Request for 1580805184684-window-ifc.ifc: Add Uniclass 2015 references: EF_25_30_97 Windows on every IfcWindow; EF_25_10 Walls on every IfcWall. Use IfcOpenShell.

First a look at what the model holds.

```python
import ifcopenshell

model = ifcopenshell.open("1580805184684-window-ifc.ifc")
print(model.schema)
print("classifications:", [c.Name for c in model.by_type("IfcClassification")])
for ifc_class in ("IfcDoor", "IfcRoof", "IfcStair", "IfcWall", "IfcWindow"):
    print(ifc_class, len(model.by_type(ifc_class)))
```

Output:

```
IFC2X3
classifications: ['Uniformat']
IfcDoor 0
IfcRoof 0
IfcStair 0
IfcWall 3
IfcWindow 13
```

```python
import ifcopenshell
import ifcopenshell.api.classification

model = ifcopenshell.open("1580805184684-window-ifc.ifc")

# IFC2X3 requires Source and Edition and has no link from the project to the system.
system = model.create_entity("IfcClassification", Source="NBS", Edition="2015", Name="Uniclass 2015")

codes = {
    "IfcWindow": ("EF_25_30_97", "Windows"),
    "IfcWall": ("EF_25_10", "Walls"),
}
for ifc_class, (code, name) in codes.items():
    products = model.by_type(ifc_class)
    ifcopenshell.api.classification.add_reference(
        model, products=products, classification=system, identification=code, name=name
    )
    print(code, len(products))

model.write("1580805184684-window-ifc-out.ifc")
```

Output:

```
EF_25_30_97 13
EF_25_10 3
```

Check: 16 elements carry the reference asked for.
